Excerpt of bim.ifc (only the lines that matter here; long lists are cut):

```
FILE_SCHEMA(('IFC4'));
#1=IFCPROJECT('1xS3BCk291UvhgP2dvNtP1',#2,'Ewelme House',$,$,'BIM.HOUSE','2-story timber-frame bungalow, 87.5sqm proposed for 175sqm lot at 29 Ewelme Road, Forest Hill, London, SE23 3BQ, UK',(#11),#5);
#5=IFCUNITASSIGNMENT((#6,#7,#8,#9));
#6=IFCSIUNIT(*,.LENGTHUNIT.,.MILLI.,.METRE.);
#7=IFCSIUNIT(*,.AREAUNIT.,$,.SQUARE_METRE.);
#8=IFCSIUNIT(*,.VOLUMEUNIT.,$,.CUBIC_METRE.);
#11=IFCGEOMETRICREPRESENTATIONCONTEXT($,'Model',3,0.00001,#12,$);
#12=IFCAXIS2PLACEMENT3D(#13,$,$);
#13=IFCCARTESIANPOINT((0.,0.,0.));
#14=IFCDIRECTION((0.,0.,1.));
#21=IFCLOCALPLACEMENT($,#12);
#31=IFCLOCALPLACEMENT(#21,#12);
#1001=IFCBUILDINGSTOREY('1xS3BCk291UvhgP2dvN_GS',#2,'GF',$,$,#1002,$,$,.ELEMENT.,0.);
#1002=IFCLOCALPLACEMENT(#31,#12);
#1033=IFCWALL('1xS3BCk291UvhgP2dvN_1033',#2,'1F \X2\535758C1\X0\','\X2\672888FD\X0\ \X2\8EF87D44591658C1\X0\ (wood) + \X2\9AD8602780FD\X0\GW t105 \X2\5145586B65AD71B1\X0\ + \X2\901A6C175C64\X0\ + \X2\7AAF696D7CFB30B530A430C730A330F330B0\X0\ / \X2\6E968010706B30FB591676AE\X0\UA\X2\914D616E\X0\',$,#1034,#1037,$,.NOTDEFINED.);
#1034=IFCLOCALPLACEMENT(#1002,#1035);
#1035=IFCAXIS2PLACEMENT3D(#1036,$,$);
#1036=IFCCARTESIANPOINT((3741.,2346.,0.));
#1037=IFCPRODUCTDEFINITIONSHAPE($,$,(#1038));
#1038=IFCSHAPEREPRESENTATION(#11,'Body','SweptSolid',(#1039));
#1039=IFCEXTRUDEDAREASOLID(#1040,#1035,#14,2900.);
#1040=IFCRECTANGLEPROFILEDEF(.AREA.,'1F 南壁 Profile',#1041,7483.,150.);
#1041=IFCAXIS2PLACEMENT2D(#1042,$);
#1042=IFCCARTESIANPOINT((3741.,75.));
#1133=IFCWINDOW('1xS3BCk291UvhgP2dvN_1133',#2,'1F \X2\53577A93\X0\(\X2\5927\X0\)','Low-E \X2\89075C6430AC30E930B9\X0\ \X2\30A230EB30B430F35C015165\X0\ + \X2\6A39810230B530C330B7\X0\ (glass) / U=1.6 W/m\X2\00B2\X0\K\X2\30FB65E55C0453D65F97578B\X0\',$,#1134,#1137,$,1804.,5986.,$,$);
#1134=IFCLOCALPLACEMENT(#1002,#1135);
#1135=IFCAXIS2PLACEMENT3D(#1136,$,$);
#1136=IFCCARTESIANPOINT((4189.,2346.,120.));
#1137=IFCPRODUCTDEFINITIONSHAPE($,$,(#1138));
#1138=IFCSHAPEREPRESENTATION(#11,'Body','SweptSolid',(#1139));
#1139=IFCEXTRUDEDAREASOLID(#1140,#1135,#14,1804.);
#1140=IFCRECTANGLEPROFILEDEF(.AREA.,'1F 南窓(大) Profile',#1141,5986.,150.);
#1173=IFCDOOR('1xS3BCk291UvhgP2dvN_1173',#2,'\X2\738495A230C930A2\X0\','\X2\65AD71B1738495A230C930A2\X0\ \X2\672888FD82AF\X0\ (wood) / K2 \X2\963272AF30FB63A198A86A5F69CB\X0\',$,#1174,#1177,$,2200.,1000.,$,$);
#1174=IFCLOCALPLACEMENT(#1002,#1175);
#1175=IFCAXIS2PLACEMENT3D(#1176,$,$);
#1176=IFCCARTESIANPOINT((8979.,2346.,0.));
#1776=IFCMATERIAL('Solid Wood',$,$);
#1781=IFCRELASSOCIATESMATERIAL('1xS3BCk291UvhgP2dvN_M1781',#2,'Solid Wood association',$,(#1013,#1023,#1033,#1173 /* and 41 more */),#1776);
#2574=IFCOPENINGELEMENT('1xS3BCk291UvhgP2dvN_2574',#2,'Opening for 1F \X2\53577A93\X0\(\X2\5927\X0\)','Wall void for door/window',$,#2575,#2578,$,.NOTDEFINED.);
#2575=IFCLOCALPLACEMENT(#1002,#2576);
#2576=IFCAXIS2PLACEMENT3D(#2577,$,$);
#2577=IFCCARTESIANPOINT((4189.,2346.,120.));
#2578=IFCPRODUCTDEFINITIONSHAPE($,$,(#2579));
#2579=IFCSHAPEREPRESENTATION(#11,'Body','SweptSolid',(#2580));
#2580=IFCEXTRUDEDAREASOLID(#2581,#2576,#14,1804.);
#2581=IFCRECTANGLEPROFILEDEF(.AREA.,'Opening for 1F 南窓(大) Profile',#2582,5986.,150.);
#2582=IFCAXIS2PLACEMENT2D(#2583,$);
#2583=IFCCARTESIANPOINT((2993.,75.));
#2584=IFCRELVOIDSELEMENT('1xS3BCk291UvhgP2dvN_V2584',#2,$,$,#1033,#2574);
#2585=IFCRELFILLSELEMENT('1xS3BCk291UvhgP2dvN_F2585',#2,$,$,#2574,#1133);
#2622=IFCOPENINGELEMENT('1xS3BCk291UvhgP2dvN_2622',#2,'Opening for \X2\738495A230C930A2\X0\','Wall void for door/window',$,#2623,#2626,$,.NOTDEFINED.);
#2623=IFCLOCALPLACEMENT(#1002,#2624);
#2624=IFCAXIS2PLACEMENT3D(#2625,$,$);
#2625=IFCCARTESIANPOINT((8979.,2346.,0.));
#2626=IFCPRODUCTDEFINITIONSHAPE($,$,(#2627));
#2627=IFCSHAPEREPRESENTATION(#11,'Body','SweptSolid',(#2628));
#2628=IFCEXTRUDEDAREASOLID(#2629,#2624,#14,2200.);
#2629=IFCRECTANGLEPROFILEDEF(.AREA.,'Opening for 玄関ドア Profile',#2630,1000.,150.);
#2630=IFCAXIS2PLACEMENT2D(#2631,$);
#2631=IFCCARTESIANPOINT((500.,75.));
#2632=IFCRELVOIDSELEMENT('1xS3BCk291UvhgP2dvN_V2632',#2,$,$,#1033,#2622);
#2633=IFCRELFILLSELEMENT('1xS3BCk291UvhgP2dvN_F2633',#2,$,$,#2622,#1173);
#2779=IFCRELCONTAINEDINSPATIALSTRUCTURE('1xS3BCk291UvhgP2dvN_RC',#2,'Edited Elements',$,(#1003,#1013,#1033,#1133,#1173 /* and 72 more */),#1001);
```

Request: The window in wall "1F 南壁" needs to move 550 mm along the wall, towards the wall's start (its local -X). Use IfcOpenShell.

```python
import ifcopenshell
import ifcopenshell.api.geometry
import ifcopenshell.util.placement
import ifcopenshell.util.unit

model = ifcopenshell.open("bim.ifc")
unit_scale = ifcopenshell.util.unit.calculate_unit_scale(model)

window = model.by_guid("1xS3BCk291UvhgP2dvN_1133")
opening = window.FillsVoids[0].RelatingOpeningElement
wall = opening.VoidsElements[0].RelatingBuildingElement

wall_matrix = ifcopenshell.util.placement.get_local_placement(wall.ObjectPlacement)
shift = wall_matrix[:3, 0] * -0.55 / unit_scale
before = ifcopenshell.util.placement.get_local_placement(window.ObjectPlacement)[:3, 3].copy()

# The window is not placed relative to its opening, so move both.
for product in (opening, window):
    matrix = ifcopenshell.util.placement.get_local_placement(product.ObjectPlacement)
    matrix[:3, 3] += shift
    ifcopenshell.api.geometry.edit_object_placement(model, product=product, matrix=matrix, is_si=False)

after = ifcopenshell.util.placement.get_local_placement(window.ObjectPlacement)[:3, 3]
print("window moved by", (after - before).round(3) + 0.0)

model.write("bim_v2.ifc")
```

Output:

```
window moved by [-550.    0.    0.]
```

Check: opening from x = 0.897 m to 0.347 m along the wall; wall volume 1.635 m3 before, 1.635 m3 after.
